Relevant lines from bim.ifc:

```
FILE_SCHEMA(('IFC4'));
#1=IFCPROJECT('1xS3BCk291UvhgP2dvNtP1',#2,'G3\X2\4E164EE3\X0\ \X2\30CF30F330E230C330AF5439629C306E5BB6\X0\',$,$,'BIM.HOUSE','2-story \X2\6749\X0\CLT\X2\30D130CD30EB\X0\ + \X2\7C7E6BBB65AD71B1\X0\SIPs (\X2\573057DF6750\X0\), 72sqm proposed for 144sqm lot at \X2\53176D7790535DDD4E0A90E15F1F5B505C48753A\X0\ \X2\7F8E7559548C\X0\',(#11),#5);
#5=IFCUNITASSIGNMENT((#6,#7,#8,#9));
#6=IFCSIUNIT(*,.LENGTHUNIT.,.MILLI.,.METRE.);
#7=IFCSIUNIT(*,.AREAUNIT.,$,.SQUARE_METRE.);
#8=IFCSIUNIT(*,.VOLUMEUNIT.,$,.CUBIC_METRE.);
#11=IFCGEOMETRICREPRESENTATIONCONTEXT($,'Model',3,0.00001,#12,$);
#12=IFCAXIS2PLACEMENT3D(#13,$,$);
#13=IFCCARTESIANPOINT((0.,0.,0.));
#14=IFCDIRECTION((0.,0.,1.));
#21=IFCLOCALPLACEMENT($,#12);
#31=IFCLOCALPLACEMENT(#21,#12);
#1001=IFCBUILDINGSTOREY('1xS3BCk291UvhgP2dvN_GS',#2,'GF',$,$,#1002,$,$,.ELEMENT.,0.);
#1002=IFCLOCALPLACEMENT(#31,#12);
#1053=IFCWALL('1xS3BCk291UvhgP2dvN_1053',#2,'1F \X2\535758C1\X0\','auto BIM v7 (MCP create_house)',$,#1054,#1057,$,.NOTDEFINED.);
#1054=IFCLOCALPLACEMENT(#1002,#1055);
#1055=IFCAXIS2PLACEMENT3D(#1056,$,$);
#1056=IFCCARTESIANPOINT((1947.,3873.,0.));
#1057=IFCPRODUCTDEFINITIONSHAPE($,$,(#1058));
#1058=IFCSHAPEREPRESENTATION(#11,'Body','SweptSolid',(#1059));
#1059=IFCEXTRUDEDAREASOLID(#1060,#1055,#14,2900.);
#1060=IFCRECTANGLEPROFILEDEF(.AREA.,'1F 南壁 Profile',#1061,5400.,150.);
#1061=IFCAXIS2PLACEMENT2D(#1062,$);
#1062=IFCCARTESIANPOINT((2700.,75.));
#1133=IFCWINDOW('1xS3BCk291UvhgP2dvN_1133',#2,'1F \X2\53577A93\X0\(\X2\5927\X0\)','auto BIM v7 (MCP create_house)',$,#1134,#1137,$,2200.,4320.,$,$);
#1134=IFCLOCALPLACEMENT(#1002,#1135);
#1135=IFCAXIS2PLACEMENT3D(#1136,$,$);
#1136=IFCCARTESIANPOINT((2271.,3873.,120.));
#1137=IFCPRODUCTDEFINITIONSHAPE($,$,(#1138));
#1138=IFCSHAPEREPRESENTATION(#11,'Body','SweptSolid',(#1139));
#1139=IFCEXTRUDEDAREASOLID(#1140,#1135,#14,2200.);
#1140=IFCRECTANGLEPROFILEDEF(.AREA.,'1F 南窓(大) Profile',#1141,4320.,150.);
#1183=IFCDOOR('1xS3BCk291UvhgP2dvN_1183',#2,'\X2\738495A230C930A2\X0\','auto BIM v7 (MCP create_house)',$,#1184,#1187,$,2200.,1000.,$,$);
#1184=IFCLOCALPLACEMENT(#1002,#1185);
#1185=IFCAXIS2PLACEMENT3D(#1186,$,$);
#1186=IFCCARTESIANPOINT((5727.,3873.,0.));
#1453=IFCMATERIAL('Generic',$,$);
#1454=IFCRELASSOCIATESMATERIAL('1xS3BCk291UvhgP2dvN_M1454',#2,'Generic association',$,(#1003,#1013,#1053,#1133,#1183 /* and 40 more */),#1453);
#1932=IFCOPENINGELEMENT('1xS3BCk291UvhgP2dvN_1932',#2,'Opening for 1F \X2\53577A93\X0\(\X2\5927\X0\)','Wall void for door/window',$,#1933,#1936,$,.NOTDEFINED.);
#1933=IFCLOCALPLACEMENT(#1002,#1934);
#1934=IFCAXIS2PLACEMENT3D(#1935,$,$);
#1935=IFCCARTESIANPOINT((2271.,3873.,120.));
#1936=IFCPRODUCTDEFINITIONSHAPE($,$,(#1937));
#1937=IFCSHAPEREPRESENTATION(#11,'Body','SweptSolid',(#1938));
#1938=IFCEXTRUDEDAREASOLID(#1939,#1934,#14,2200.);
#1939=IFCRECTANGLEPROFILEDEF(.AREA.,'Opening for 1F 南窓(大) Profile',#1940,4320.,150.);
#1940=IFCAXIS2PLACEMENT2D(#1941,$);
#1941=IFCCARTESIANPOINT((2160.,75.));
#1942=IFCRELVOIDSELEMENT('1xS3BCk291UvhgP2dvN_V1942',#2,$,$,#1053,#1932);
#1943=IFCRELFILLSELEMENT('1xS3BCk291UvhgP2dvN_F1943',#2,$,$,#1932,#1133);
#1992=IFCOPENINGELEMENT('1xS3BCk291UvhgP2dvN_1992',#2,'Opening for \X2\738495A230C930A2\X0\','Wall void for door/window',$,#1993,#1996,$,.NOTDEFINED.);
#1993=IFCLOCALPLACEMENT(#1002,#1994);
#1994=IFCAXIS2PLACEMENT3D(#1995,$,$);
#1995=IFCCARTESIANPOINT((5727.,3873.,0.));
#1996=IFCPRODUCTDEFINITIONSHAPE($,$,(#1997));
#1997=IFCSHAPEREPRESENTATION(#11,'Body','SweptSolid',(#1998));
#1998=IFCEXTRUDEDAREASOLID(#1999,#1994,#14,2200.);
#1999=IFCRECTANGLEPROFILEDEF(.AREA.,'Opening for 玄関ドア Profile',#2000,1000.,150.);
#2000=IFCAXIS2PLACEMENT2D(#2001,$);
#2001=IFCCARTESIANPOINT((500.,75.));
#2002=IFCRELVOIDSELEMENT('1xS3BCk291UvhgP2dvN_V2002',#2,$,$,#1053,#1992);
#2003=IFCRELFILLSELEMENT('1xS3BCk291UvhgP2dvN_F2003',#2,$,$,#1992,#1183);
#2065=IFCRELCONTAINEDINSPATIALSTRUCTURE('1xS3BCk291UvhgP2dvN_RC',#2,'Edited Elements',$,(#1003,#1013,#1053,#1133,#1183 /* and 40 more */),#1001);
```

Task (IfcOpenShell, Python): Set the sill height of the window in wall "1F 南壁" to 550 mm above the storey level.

```python
import numpy as np
import ifcopenshell
import ifcopenshell.api.geometry
import ifcopenshell.geom
import ifcopenshell.util.element
import ifcopenshell.util.placement
import ifcopenshell.util.shape
import ifcopenshell.util.unit

model = ifcopenshell.open("bim.ifc")
unit_scale = ifcopenshell.util.unit.calculate_unit_scale(model)

window = model.by_guid("1xS3BCk291UvhgP2dvN_1133")
opening = window.FillsVoids[0].RelatingOpeningElement
storey = ifcopenshell.util.element.get_container(window, ifc_class="IfcBuildingStorey")
level = ifcopenshell.util.placement.get_local_placement(storey.ObjectPlacement)[2, 3]

# The opening's origin need not be at the sill, so measure its lowest point.
shape = ifcopenshell.geom.create_shape(ifcopenshell.geom.settings(), opening)
bottom = ifcopenshell.util.shape.get_shape_bottom_elevation(shape, shape.geometry) / unit_scale
dz = level + 0.55 / unit_scale - bottom

shift = np.array([0.0, 0.0, dz])
# The window is not placed relative to its opening, so move both.
for product in (opening, window):
    matrix = ifcopenshell.util.placement.get_local_placement(product.ObjectPlacement)
    matrix[:3, 3] += shift
    ifcopenshell.api.geometry.edit_object_placement(model, product=product, matrix=matrix, is_si=False)

print(f"moved by {dz * unit_scale:+.3f} m")

model.write("bim_edited.ifc")
```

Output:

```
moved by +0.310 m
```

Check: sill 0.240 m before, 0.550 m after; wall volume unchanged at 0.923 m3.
